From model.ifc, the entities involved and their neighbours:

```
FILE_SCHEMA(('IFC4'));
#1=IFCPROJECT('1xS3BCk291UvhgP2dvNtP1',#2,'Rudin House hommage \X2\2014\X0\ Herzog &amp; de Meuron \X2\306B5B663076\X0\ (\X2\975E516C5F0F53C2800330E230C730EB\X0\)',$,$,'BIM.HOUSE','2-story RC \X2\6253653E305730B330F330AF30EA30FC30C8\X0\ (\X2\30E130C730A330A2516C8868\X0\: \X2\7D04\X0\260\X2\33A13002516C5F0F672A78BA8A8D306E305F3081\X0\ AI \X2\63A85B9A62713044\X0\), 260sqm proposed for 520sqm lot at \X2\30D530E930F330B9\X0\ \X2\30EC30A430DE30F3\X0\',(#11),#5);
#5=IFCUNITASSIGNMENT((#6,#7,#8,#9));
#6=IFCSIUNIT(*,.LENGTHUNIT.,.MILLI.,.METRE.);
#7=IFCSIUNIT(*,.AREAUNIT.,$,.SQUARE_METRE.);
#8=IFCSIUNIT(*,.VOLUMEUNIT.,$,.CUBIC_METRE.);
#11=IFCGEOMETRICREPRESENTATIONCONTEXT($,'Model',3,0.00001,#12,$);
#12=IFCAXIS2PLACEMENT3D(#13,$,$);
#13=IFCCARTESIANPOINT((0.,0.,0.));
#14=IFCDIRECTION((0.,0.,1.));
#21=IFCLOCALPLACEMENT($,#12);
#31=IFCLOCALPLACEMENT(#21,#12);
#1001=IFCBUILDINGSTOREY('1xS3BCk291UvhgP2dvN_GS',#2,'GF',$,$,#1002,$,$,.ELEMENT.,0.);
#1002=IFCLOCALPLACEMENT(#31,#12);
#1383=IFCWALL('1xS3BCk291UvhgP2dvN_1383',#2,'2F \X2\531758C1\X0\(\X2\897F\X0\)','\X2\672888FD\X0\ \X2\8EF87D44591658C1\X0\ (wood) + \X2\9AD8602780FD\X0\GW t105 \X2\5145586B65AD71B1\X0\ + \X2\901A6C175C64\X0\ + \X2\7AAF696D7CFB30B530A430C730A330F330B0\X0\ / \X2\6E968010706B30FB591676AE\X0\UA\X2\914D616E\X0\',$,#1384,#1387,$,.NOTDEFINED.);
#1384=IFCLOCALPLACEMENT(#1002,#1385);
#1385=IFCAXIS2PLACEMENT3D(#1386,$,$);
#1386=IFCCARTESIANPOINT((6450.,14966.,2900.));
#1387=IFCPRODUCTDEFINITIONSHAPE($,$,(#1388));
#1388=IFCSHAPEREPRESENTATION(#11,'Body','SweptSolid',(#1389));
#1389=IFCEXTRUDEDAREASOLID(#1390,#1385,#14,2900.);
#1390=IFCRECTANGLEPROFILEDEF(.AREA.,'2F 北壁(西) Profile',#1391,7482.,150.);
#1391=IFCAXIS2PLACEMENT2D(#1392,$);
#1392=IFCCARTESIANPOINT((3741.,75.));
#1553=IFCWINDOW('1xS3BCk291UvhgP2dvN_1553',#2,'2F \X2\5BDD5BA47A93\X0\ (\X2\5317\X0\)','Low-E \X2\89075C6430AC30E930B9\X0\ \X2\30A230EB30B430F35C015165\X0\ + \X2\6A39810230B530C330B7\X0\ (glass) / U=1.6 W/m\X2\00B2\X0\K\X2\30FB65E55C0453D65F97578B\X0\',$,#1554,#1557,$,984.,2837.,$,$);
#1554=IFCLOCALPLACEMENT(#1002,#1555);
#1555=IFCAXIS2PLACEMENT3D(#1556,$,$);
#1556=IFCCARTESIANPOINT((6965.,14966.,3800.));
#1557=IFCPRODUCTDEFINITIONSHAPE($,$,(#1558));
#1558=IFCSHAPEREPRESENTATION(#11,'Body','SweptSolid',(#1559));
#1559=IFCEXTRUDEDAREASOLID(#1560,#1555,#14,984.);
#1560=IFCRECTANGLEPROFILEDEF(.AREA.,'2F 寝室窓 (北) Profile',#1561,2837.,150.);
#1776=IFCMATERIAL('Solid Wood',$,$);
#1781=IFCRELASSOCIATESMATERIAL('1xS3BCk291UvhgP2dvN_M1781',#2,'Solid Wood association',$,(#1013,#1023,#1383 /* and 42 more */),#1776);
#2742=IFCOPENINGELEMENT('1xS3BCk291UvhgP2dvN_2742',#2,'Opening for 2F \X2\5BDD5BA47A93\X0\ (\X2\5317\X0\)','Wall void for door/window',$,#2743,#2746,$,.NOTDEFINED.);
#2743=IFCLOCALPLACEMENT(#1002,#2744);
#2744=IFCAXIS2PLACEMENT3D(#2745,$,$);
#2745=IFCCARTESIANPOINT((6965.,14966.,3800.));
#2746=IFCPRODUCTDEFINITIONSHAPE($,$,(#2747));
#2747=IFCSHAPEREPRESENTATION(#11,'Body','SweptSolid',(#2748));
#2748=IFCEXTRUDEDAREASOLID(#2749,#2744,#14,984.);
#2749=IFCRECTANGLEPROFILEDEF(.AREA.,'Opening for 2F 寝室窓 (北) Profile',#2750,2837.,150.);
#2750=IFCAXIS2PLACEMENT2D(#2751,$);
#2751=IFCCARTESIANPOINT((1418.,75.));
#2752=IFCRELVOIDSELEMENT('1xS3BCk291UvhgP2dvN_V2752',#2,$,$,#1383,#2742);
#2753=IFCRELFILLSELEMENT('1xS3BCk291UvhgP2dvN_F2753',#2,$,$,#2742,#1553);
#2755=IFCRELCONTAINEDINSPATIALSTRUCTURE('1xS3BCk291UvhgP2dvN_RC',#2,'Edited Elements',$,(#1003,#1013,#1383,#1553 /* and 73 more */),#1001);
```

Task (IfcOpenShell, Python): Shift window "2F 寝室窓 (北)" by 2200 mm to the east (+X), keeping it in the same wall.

```python
import ifcopenshell
import ifcopenshell.api.geometry
import ifcopenshell.util.placement
import ifcopenshell.util.unit

model = ifcopenshell.open("model.ifc")
unit_scale = ifcopenshell.util.unit.calculate_unit_scale(model)

window = model.by_id(1553)
opening = window.FillsVoids[0].RelatingOpeningElement
wall = opening.VoidsElements[0].RelatingBuildingElement

wall_matrix = ifcopenshell.util.placement.get_local_placement(wall.ObjectPlacement)
shift = wall_matrix[:3, 0] * 2.2 / unit_scale
before = ifcopenshell.util.placement.get_local_placement(window.ObjectPlacement)[:3, 3].copy()

# The window is not placed relative to its opening, so move both.
for product in (opening, window):
    matrix = ifcopenshell.util.placement.get_local_placement(product.ObjectPlacement)
    matrix[:3, 3] += shift
    ifcopenshell.api.geometry.edit_object_placement(model, product=product, matrix=matrix, is_si=False)

after = ifcopenshell.util.placement.get_local_placement(window.ObjectPlacement)[:3, 3]
print("window moved by", (after - before).round(3) + 0.0)

model.write("model_updated.ifc")
```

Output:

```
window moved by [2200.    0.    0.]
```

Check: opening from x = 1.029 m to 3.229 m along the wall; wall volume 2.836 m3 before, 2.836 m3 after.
